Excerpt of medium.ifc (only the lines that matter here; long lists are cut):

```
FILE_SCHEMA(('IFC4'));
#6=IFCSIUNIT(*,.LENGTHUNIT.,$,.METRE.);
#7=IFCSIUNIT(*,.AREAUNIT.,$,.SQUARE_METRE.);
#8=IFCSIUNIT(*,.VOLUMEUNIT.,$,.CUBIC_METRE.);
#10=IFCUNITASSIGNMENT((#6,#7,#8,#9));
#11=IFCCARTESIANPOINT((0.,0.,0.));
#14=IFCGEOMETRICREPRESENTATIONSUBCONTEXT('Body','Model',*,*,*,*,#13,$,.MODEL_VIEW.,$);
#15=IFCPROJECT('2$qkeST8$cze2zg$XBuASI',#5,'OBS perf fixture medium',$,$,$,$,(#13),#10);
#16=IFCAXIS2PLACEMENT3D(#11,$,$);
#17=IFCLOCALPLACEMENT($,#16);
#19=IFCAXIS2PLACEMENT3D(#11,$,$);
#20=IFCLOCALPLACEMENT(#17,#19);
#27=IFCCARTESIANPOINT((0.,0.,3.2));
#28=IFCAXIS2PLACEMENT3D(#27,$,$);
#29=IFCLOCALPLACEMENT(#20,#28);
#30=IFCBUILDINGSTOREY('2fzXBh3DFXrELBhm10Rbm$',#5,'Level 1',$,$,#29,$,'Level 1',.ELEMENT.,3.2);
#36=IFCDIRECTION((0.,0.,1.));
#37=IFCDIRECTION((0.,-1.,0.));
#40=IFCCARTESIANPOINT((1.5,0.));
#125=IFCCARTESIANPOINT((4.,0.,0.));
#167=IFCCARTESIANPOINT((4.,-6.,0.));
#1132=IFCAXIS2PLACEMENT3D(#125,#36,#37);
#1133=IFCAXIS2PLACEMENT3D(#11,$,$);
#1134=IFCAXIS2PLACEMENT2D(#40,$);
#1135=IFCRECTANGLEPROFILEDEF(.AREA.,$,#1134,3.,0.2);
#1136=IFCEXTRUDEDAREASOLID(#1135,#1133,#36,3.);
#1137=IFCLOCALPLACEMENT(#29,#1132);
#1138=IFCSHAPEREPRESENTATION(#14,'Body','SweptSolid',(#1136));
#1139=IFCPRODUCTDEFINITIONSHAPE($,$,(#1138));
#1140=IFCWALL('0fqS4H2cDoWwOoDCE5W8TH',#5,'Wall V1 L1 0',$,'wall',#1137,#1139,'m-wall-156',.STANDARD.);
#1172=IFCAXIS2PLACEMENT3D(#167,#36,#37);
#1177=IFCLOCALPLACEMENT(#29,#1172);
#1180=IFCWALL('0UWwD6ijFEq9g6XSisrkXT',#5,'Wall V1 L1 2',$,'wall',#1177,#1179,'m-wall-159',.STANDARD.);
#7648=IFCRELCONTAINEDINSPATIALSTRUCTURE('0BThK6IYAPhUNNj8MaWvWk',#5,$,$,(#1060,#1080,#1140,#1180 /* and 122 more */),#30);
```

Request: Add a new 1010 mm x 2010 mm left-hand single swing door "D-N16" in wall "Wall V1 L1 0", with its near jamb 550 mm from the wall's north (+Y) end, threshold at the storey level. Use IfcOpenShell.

```python
import numpy as np
import ifcopenshell
import ifcopenshell.api.feature
import ifcopenshell.api.geometry
import ifcopenshell.api.root
import ifcopenshell.api.spatial
import ifcopenshell.geom
import ifcopenshell.util.element
import ifcopenshell.util.placement
import ifcopenshell.util.representation
import ifcopenshell.util.shape
import ifcopenshell.util.unit

model = ifcopenshell.open("medium.ifc")
unit_scale = ifcopenshell.util.unit.calculate_unit_scale(model)
settings = ifcopenshell.geom.settings()


def volume(element):
    """Net volume in cubic metres, openings subtracted."""
    shape = ifcopenshell.geom.create_shape(settings, element)
    return ifcopenshell.util.shape.get_volume(shape.geometry)


wall = model.by_guid("0fqS4H2cDoWwOoDCE5W8TH")
storey = ifcopenshell.util.element.get_container(wall, ifc_class="IfcBuildingStorey")
context = ifcopenshell.util.representation.get_context(model, "Model", "Body", "MODEL_VIEW")
before = volume(wall)

width, height, from_end, sill = 1.01, 2.01, 0.55, 0.0  # metres

# The wall runs along its own X axis, and the end named is its -X end.
wall_shape = ifcopenshell.geom.create_shape(settings, wall)
x, y, z = ifcopenshell.util.shape.get_vertices(wall_shape.geometry).T
start = x.min() + from_end
face, thickness = float(y.min()), float(y.max() - y.min())
wall_matrix = ifcopenshell.util.placement.get_local_placement(wall.ObjectPlacement)
level = ifcopenshell.util.placement.get_local_placement(storey.ObjectPlacement)[2, 3]


def in_wall(x, y):
    """Placement at x, y metres in the wall's axes, at sill height."""
    matrix = wall_matrix.copy()
    matrix[:, 3] = wall_matrix @ np.array([x / unit_scale, y / unit_scale, 0.0, 1.0])
    matrix[2, 3] = level + sill / unit_scale
    return matrix


# Opening: a box that overshoots both wall faces by 50 mm.
opening = ifcopenshell.api.root.create_entity(model, ifc_class="IfcOpeningElement", predefined_type="OPENING")
box = ifcopenshell.api.geometry.add_wall_representation(
    model, context=context, length=width, height=height, thickness=thickness + 0.1
)
ifcopenshell.api.geometry.assign_representation(model, product=opening, representation=box)
ifcopenshell.api.geometry.edit_object_placement(model, product=opening, matrix=in_wall(start, face - 0.05), is_si=False)
ifcopenshell.api.feature.add_feature(model, feature=opening, element=wall)

door = ifcopenshell.api.root.create_entity(model, ifc_class="IfcDoor", name="D-N16", predefined_type="DOOR")
door.OverallWidth, door.OverallHeight = width / unit_scale, height / unit_scale
door.OperationType = "SINGLE_SWING_LEFT"
body = ifcopenshell.api.geometry.add_door_representation(
    model,
    context=context,
    overall_width=door.OverallWidth,
    overall_height=door.OverallHeight,
    operation_type="SINGLE_SWING_LEFT",
    lining_properties={"LiningDepth": thickness / unit_scale, "ThresholdDepth": thickness / unit_scale},
)
ifcopenshell.api.geometry.assign_representation(model, product=door, representation=body)
ifcopenshell.api.spatial.assign_container(model, products=[door], relating_structure=storey)
ifcopenshell.api.feature.add_filling(model, opening=opening, element=door)

# The lining spans the wall, so the door starts at the wall face.
ifcopenshell.api.geometry.edit_object_placement(model, product=door, matrix=in_wall(start, face), is_si=False)

after = volume(wall)

print(f"wall volume {before:.3f} -> {after:.3f} m3")

model.write("medium_edited.ifc")
```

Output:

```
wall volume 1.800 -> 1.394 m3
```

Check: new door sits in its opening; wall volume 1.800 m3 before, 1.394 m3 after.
